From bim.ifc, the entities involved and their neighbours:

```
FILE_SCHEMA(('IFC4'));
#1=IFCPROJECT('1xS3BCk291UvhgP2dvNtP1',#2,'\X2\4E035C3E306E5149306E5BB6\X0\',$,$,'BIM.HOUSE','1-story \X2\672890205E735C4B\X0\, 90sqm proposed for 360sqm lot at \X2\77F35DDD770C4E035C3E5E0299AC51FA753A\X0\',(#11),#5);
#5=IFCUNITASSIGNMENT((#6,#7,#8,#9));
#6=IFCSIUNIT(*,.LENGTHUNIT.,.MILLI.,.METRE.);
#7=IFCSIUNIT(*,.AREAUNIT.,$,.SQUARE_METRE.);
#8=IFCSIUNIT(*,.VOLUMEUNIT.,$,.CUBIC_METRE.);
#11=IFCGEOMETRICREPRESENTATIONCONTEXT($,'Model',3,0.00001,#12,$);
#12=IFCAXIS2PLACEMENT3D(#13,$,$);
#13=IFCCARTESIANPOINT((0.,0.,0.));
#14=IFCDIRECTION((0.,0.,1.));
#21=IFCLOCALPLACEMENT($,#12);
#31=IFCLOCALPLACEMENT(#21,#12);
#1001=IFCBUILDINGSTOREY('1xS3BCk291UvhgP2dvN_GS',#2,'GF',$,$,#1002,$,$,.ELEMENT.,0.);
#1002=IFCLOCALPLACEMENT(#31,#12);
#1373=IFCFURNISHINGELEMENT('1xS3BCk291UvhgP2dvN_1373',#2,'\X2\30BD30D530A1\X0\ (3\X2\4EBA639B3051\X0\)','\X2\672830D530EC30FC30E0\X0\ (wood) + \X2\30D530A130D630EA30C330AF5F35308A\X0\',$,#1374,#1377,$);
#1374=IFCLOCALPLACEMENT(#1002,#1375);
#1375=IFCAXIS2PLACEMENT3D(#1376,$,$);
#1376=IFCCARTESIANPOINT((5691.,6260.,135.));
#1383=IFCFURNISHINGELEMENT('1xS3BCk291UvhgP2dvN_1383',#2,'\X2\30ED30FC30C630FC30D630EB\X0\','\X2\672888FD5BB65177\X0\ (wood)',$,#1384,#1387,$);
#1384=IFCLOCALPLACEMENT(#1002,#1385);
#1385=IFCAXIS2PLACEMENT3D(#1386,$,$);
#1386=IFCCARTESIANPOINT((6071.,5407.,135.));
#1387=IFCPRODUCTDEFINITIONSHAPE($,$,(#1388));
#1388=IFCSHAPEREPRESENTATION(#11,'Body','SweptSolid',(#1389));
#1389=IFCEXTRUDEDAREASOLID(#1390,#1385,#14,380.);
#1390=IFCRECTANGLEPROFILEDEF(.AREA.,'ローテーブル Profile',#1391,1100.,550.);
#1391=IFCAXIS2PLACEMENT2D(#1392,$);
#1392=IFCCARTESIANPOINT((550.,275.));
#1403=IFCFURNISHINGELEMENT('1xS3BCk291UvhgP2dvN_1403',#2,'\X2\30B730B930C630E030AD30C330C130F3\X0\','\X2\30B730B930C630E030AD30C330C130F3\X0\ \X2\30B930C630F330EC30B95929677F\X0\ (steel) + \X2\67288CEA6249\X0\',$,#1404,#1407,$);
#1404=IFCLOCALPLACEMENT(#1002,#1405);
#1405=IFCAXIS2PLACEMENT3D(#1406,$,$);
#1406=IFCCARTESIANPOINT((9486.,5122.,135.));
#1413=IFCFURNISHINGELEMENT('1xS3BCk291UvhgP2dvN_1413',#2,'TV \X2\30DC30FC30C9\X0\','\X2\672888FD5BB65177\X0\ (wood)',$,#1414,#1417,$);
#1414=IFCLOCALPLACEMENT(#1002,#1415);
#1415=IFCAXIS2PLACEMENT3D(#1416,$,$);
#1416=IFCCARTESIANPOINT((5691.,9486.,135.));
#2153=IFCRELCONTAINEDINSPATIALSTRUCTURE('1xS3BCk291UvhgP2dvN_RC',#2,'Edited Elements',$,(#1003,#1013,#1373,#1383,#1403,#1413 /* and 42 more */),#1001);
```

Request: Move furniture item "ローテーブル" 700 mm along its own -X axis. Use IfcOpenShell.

```python
import ifcopenshell
import ifcopenshell.api.geometry
import ifcopenshell.util.placement

model = ifcopenshell.open("bim.ifc")

item = model.by_guid("1xS3BCk291UvhgP2dvN_1383")
matrix = ifcopenshell.util.placement.get_local_placement(item.ObjectPlacement)
matrix[:3, 3] -= matrix[:3, 0] * 700.0
ifcopenshell.api.geometry.edit_object_placement(model, product=item, matrix=matrix, is_si=False)

print(ifcopenshell.util.placement.get_local_placement(item.ObjectPlacement).round(3) + 0.0)

model.write("bim_updated.ifc")
```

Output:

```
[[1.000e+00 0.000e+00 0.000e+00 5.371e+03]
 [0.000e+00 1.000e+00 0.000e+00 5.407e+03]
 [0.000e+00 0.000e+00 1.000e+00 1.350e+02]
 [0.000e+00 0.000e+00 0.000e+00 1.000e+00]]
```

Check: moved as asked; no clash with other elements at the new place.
